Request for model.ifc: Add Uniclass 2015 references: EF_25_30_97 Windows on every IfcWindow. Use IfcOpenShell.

First a look at what the model holds.

```python
import ifcopenshell

model = ifcopenshell.open("model.ifc")
print(model.schema)
print("classifications:", [c.Name for c in model.by_type("IfcClassification")])
for ifc_class in ("IfcDoor", "IfcRoof", "IfcStair", "IfcWall", "IfcWindow"):
    print(ifc_class, len(model.by_type(ifc_class)))
```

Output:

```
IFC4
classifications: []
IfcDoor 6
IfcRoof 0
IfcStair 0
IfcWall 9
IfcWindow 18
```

```python
import ifcopenshell
import ifcopenshell.api.classification

model = ifcopenshell.open("model.ifc")

system = ifcopenshell.api.classification.add_classification(model, classification="Uniclass 2015")

codes = {
    "IfcWindow": ("EF_25_30_97", "Windows"),
}
for ifc_class, (code, name) in codes.items():
    products = model.by_type(ifc_class)
    ifcopenshell.api.classification.add_reference(
        model, products=products, classification=system, identification=code, name=name
    )
    print(code, len(products))

model.write("model_rev.ifc")
```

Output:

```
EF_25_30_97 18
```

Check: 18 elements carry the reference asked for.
